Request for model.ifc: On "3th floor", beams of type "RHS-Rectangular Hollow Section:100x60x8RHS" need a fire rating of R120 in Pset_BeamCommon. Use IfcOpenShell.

First a look at what the model holds.

```python
import ifcopenshell
import ifcopenshell.util.element

model = ifcopenshell.open("model.ifc")
print(model.schema)
storey = next(s for s in model.by_type("IfcBuildingStorey") if s.Name == "3th floor")
beams = [e for e in ifcopenshell.util.element.get_decomposition(storey) if e.is_a("IfcBeam")]
seen = {}
for e in beams:
    element_type = ifcopenshell.util.element.get_type(e)
    key = (element_type.Name if element_type != e and element_type else None, ifcopenshell.util.element.get_pset(e, "Pset_BeamCommon", "FireRating"))
    seen[key] = seen.get(key, 0) + 1
for (name, value), count in sorted(seen.items(), key=str):
    print(count, "x", name, "|", value)
```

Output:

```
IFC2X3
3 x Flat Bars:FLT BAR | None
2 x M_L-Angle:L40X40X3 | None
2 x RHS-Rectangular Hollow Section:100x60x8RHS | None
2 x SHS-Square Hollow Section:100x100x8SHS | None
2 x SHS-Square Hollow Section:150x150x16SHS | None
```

```python
import ifcopenshell
import ifcopenshell.api.pset
import ifcopenshell.util.element

model = ifcopenshell.open("model.ifc")

storey = next(s for s in model.by_type("IfcBuildingStorey") if s.Name == "3th floor")
beams = [e for e in ifcopenshell.util.element.get_decomposition(storey) if e.is_a("IfcBeam")]

count = 0
for e in beams:
    element_type = ifcopenshell.util.element.get_type(e)
    if element_type in (None, e) or element_type.Name != "RHS-Rectangular Hollow Section:100x60x8RHS":
        continue
    # add_pset returns the element's existing set when there is one.
    pset = ifcopenshell.api.pset.add_pset(model, product=e, name="Pset_BeamCommon")
    ifcopenshell.api.pset.edit_pset(model, pset=pset, properties={"FireRating": "R120"})
    count += 1

print(count, "beams updated")

model.write("model-out.ifc")
```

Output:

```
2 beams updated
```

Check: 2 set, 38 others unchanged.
